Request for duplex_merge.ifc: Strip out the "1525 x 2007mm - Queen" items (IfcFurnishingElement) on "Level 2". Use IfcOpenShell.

First a look at what the model holds.

```python
import ifcopenshell
import ifcopenshell.util.element

model = ifcopenshell.open("duplex_merge.ifc")
print(model.schema)
storey = next(s for s in model.by_type("IfcBuildingStorey") if s.Name == "Level 2")
furniture = [e for e in ifcopenshell.util.element.get_decomposition(storey) if e.is_a("IfcFurnishingElement")]
seen = {}
for e in furniture:
    element_type = ifcopenshell.util.element.get_type(e)
    name = element_type.Name if element_type not in (None, e) else None
    seen[name] = seen.get(name, 0) + 1
for name, count in sorted(seen.items(), key=str):
    print(count, "x", name)
```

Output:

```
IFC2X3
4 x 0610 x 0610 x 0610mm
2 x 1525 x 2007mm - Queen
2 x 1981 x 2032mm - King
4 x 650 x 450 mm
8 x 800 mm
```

```python
import ifcopenshell
import ifcopenshell.api.root
import ifcopenshell.util.element

model = ifcopenshell.open("duplex_merge.ifc")

storey = next(s for s in model.by_type("IfcBuildingStorey") if s.Name == "Level 2")
furniture = [e for e in ifcopenshell.util.element.get_decomposition(storey) if e.is_a("IfcFurnishingElement")]
targets = [e for e in furniture if (t := ifcopenshell.util.element.get_type(e)) not in (None, e) and t.Name == "1525 x 2007mm - Queen"]

for e in targets:
    ifcopenshell.api.root.remove_product(model, product=e)
print(len(targets), "removed")

model.write("duplex_merge_v2.ifc")
```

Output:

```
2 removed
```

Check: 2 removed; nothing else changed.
